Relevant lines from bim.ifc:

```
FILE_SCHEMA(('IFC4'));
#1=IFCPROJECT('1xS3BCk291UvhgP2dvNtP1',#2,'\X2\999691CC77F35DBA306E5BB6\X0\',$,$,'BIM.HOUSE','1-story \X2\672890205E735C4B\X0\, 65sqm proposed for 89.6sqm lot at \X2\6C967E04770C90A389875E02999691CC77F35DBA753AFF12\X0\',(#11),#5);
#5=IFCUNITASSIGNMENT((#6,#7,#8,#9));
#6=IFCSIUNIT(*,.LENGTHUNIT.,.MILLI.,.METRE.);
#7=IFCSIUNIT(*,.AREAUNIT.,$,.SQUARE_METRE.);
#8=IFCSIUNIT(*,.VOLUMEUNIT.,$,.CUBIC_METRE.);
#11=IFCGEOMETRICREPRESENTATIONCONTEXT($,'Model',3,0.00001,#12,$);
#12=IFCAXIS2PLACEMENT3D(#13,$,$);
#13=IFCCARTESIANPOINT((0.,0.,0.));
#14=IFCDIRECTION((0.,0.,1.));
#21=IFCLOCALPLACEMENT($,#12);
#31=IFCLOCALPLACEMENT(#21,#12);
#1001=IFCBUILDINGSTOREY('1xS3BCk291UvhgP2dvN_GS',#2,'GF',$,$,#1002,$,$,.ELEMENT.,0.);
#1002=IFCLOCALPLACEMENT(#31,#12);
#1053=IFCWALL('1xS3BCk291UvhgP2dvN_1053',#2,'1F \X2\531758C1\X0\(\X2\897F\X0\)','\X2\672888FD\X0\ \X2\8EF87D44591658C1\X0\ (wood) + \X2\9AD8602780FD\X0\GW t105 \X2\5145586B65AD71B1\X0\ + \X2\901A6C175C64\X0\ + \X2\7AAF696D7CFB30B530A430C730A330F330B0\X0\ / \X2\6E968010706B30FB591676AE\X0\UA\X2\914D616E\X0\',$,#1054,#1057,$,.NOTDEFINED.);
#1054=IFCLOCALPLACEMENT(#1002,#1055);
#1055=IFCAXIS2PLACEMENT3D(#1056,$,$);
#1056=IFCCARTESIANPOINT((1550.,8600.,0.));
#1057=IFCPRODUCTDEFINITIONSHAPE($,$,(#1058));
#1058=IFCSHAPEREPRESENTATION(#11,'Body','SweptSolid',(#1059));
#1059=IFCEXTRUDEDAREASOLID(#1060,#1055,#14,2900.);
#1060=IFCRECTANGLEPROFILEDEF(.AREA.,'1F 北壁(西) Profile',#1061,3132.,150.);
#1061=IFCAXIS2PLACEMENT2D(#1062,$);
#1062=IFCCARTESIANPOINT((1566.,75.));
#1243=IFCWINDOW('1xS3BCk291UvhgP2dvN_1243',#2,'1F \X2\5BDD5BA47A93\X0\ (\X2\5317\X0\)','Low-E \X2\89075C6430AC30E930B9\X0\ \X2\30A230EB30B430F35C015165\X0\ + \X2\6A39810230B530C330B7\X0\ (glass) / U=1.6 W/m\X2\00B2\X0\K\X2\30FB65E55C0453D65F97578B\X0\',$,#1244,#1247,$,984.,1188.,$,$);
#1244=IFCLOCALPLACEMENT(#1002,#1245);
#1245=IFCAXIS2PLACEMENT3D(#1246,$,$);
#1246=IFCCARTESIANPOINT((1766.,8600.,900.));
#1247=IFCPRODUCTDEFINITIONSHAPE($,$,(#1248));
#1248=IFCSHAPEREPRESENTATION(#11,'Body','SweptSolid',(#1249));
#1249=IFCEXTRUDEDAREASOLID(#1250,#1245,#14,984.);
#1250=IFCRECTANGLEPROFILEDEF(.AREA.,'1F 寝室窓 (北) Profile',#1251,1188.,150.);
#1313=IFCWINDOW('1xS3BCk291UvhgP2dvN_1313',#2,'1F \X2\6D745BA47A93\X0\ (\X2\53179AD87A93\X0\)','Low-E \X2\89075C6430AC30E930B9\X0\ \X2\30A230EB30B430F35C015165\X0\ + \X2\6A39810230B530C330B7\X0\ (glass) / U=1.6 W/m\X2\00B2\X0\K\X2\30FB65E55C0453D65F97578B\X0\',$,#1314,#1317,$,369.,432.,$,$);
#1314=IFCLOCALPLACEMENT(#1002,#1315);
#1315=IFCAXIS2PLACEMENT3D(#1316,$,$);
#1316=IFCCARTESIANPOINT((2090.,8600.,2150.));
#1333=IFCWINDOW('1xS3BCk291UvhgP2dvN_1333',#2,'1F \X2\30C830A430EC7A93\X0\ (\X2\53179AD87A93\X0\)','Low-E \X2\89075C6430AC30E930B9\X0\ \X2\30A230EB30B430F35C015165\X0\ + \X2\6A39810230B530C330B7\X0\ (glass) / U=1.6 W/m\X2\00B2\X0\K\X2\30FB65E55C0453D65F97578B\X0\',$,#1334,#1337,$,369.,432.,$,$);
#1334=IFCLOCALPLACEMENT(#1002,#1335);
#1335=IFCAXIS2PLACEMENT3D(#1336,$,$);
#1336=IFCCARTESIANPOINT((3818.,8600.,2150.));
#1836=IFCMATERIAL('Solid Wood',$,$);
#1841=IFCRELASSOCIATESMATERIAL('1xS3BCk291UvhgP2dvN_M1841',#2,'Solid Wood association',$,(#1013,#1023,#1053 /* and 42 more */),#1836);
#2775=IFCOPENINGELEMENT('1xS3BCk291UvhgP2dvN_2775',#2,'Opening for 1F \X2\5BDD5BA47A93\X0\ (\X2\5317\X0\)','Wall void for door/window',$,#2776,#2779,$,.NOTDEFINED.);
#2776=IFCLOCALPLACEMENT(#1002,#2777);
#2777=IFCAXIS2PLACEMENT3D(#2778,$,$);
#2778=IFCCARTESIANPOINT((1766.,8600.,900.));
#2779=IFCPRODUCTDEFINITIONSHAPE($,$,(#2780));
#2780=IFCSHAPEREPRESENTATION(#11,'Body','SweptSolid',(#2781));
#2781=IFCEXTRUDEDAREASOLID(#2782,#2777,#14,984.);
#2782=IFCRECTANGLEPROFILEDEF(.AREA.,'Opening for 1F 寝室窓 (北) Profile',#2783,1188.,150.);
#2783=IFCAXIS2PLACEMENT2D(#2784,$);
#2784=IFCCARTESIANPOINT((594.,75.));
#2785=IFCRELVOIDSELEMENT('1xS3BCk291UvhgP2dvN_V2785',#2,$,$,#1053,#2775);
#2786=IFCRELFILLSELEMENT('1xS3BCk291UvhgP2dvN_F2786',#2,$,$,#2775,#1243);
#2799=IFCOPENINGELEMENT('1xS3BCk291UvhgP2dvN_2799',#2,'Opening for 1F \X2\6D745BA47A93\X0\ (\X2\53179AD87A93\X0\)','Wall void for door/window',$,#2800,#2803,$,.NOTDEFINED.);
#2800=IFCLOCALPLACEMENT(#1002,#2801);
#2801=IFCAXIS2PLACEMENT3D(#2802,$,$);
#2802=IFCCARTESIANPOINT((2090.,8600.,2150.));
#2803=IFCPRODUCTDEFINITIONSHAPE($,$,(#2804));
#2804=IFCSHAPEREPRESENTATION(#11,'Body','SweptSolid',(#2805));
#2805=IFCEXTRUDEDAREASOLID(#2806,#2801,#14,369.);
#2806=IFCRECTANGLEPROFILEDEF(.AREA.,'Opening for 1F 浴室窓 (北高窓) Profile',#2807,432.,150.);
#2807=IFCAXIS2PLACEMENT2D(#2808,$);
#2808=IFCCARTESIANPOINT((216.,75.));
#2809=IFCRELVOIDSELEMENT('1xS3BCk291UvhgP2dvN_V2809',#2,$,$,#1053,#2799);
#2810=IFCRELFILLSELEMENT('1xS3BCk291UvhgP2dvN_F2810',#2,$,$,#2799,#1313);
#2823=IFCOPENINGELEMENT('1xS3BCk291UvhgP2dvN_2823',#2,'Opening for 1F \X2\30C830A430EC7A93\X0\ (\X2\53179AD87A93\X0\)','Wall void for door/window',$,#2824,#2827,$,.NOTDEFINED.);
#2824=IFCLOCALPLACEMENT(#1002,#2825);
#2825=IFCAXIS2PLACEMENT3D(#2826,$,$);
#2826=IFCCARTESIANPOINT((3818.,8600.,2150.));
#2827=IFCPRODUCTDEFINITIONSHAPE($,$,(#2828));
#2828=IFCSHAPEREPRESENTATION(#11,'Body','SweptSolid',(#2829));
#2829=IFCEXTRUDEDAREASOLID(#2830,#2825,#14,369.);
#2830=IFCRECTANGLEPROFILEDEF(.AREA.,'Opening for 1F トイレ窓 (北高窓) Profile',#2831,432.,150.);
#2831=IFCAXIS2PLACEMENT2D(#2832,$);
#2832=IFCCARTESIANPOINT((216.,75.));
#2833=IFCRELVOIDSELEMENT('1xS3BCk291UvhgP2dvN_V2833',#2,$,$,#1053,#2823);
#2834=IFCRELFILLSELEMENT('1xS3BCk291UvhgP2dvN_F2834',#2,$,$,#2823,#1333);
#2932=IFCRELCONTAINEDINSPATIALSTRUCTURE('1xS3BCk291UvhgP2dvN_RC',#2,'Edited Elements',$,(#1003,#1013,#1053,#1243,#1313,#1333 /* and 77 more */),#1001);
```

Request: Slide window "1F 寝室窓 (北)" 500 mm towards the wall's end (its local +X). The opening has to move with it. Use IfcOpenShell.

```python
import ifcopenshell
import ifcopenshell.api.geometry
import ifcopenshell.util.placement
import ifcopenshell.util.unit

model = ifcopenshell.open("bim.ifc")
unit_scale = ifcopenshell.util.unit.calculate_unit_scale(model)

window = model.by_guid("1xS3BCk291UvhgP2dvN_1243")
opening = window.FillsVoids[0].RelatingOpeningElement
wall = opening.VoidsElements[0].RelatingBuildingElement

wall_matrix = ifcopenshell.util.placement.get_local_placement(wall.ObjectPlacement)
shift = wall_matrix[:3, 0] * 0.5 / unit_scale
before = ifcopenshell.util.placement.get_local_placement(window.ObjectPlacement)[:3, 3].copy()

# The window is not placed relative to its opening, so move both.
for product in (opening, window):
    matrix = ifcopenshell.util.placement.get_local_placement(product.ObjectPlacement)
    matrix[:3, 3] += shift
    ifcopenshell.api.geometry.edit_object_placement(model, product=product, matrix=matrix, is_si=False)

after = ifcopenshell.util.placement.get_local_placement(window.ObjectPlacement)[:3, 3]
print("window moved by", (after - before).round(3) + 0.0)

model.write("bim_updated.ifc")
```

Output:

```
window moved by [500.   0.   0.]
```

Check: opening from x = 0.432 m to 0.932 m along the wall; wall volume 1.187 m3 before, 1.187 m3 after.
